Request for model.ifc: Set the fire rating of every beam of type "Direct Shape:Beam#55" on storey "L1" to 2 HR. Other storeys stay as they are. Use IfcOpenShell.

First a look at what the model holds.

```python
import ifcopenshell
import ifcopenshell.util.element

model = ifcopenshell.open("model.ifc")
print(model.schema)
storey = next(s for s in model.by_type("IfcBuildingStorey") if s.Name == "L1")
beams = [e for e in ifcopenshell.util.element.get_decomposition(storey) if e.is_a("IfcBeam")]
seen = {}
for e in beams:
    element_type = ifcopenshell.util.element.get_type(e)
    key = (element_type.Name if element_type != e and element_type else None, ifcopenshell.util.element.get_pset(e, "Pset_BeamCommon", "FireRating"))
    seen[key] = seen.get(key, 0) + 1
for (name, value), count in sorted(seen.items(), key=str):
    print(count, "x", name, "|", value)
```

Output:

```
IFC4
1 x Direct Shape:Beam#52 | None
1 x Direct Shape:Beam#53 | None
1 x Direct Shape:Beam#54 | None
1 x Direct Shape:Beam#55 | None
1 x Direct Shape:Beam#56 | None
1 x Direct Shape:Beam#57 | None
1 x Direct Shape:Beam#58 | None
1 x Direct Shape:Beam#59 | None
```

```python
import ifcopenshell
import ifcopenshell.api.pset
import ifcopenshell.util.element

model = ifcopenshell.open("model.ifc")

storey = next(s for s in model.by_type("IfcBuildingStorey") if s.Name == "L1")
beams = [e for e in ifcopenshell.util.element.get_decomposition(storey) if e.is_a("IfcBeam")]

count = 0
for e in beams:
    element_type = ifcopenshell.util.element.get_type(e)
    if element_type in (None, e) or element_type.Name != "Direct Shape:Beam#55":
        continue
    # add_pset returns the element's existing set when there is one.
    pset = ifcopenshell.api.pset.add_pset(model, product=e, name="Pset_BeamCommon")
    ifcopenshell.api.pset.edit_pset(model, pset=pset, properties={"FireRating": "2 HR"})
    count += 1

print(count, "beams updated")

model.write("model_edited.ifc")
```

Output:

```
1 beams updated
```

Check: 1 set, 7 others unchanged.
